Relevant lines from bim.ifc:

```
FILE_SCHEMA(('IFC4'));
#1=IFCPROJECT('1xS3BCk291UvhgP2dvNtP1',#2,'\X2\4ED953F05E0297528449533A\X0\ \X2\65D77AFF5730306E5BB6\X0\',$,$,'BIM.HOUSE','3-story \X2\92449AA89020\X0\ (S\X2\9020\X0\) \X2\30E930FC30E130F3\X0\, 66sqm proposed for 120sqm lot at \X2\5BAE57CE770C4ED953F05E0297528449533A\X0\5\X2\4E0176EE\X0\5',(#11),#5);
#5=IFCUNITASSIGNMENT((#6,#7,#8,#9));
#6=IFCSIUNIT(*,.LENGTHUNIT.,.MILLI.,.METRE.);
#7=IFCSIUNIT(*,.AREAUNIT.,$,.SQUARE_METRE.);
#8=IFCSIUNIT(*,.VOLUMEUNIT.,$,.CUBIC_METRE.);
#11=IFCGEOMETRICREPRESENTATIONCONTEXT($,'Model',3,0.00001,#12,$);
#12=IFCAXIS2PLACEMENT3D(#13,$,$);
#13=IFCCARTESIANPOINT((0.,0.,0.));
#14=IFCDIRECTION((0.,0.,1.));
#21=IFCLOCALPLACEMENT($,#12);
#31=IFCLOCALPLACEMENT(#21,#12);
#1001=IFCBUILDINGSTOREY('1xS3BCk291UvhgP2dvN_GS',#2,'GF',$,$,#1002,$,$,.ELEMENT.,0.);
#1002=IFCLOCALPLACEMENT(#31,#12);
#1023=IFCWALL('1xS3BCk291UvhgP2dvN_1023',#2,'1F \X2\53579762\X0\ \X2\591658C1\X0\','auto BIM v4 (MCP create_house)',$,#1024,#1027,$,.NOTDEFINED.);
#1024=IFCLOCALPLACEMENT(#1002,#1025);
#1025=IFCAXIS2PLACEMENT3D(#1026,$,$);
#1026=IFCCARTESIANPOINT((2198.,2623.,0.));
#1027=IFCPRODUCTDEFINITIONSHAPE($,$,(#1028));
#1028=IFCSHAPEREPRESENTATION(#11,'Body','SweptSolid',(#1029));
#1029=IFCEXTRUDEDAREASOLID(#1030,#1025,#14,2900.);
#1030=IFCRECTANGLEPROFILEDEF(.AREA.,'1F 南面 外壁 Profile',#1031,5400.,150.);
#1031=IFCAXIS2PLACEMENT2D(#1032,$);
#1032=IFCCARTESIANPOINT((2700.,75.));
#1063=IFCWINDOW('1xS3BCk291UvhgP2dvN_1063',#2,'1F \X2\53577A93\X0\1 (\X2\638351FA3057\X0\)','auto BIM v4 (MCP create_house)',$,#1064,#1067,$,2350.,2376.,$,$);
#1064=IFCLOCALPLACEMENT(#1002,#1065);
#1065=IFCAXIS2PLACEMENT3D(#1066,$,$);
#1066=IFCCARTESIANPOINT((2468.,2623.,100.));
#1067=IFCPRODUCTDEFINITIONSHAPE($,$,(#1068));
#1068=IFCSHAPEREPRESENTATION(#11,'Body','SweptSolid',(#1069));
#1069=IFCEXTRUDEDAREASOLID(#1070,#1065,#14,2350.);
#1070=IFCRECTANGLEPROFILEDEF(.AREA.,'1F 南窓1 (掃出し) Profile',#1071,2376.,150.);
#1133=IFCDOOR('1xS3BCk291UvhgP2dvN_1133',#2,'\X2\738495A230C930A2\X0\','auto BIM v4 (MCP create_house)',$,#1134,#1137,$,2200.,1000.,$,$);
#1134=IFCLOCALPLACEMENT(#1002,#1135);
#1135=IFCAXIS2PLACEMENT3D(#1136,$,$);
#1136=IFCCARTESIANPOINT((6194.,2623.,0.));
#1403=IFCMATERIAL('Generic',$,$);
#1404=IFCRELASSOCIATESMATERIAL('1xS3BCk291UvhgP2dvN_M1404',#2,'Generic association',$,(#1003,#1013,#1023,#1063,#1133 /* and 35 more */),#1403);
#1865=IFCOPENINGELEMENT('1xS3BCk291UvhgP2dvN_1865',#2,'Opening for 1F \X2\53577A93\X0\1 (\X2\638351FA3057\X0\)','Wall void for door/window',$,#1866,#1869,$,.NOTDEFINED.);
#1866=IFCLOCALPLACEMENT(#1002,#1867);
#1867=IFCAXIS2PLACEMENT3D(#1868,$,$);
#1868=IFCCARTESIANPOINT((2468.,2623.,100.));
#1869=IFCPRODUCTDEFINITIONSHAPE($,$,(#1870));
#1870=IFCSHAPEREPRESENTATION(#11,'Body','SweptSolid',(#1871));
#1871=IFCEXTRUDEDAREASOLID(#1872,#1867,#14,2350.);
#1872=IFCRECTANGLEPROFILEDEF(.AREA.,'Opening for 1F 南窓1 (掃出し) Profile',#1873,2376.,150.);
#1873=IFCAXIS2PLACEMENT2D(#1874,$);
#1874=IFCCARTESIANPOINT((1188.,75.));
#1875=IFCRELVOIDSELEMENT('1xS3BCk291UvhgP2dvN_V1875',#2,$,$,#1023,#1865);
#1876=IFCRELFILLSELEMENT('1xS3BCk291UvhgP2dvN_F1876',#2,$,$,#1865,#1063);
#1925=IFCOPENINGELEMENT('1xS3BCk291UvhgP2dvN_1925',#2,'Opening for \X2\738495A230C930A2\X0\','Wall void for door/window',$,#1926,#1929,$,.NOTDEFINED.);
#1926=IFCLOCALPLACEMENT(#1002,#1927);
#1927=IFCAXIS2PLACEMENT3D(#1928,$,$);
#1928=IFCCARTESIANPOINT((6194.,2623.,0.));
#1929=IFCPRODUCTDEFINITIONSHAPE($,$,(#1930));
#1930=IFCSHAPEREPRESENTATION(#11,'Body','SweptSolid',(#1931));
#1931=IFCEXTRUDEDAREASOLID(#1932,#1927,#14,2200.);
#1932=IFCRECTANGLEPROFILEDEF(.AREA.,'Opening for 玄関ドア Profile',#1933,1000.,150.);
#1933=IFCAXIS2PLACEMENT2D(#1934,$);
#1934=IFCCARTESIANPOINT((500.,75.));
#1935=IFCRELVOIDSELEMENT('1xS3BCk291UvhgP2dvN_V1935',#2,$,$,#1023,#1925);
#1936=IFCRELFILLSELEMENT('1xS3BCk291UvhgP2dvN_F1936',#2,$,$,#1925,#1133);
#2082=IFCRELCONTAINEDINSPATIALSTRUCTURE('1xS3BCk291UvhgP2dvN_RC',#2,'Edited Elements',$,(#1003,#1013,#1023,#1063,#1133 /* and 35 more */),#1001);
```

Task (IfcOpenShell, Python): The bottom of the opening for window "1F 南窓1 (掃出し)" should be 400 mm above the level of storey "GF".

```python
import numpy as np
import ifcopenshell
import ifcopenshell.api.geometry
import ifcopenshell.geom
import ifcopenshell.util.element
import ifcopenshell.util.placement
import ifcopenshell.util.shape
import ifcopenshell.util.unit

model = ifcopenshell.open("bim.ifc")
unit_scale = ifcopenshell.util.unit.calculate_unit_scale(model)

window = model.by_guid("1xS3BCk291UvhgP2dvN_1063")
opening = window.FillsVoids[0].RelatingOpeningElement
storey = ifcopenshell.util.element.get_container(window, ifc_class="IfcBuildingStorey")
level = ifcopenshell.util.placement.get_local_placement(storey.ObjectPlacement)[2, 3]

# The opening's origin need not be at the sill, so measure its lowest point.
shape = ifcopenshell.geom.create_shape(ifcopenshell.geom.settings(), opening)
bottom = ifcopenshell.util.shape.get_shape_bottom_elevation(shape, shape.geometry) / unit_scale
dz = level + 400.0 - bottom

shift = np.array([0.0, 0.0, dz])
# The window is not placed relative to its opening, so move both.
for product in (opening, window):
    matrix = ifcopenshell.util.placement.get_local_placement(product.ObjectPlacement)
    matrix[:3, 3] += shift
    ifcopenshell.api.geometry.edit_object_placement(model, product=product, matrix=matrix, is_si=False)

print(f"moved by {dz * unit_scale:+.3f} m")

model.write("bim-out.ifc")
```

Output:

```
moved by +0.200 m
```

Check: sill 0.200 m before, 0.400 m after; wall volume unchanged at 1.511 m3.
